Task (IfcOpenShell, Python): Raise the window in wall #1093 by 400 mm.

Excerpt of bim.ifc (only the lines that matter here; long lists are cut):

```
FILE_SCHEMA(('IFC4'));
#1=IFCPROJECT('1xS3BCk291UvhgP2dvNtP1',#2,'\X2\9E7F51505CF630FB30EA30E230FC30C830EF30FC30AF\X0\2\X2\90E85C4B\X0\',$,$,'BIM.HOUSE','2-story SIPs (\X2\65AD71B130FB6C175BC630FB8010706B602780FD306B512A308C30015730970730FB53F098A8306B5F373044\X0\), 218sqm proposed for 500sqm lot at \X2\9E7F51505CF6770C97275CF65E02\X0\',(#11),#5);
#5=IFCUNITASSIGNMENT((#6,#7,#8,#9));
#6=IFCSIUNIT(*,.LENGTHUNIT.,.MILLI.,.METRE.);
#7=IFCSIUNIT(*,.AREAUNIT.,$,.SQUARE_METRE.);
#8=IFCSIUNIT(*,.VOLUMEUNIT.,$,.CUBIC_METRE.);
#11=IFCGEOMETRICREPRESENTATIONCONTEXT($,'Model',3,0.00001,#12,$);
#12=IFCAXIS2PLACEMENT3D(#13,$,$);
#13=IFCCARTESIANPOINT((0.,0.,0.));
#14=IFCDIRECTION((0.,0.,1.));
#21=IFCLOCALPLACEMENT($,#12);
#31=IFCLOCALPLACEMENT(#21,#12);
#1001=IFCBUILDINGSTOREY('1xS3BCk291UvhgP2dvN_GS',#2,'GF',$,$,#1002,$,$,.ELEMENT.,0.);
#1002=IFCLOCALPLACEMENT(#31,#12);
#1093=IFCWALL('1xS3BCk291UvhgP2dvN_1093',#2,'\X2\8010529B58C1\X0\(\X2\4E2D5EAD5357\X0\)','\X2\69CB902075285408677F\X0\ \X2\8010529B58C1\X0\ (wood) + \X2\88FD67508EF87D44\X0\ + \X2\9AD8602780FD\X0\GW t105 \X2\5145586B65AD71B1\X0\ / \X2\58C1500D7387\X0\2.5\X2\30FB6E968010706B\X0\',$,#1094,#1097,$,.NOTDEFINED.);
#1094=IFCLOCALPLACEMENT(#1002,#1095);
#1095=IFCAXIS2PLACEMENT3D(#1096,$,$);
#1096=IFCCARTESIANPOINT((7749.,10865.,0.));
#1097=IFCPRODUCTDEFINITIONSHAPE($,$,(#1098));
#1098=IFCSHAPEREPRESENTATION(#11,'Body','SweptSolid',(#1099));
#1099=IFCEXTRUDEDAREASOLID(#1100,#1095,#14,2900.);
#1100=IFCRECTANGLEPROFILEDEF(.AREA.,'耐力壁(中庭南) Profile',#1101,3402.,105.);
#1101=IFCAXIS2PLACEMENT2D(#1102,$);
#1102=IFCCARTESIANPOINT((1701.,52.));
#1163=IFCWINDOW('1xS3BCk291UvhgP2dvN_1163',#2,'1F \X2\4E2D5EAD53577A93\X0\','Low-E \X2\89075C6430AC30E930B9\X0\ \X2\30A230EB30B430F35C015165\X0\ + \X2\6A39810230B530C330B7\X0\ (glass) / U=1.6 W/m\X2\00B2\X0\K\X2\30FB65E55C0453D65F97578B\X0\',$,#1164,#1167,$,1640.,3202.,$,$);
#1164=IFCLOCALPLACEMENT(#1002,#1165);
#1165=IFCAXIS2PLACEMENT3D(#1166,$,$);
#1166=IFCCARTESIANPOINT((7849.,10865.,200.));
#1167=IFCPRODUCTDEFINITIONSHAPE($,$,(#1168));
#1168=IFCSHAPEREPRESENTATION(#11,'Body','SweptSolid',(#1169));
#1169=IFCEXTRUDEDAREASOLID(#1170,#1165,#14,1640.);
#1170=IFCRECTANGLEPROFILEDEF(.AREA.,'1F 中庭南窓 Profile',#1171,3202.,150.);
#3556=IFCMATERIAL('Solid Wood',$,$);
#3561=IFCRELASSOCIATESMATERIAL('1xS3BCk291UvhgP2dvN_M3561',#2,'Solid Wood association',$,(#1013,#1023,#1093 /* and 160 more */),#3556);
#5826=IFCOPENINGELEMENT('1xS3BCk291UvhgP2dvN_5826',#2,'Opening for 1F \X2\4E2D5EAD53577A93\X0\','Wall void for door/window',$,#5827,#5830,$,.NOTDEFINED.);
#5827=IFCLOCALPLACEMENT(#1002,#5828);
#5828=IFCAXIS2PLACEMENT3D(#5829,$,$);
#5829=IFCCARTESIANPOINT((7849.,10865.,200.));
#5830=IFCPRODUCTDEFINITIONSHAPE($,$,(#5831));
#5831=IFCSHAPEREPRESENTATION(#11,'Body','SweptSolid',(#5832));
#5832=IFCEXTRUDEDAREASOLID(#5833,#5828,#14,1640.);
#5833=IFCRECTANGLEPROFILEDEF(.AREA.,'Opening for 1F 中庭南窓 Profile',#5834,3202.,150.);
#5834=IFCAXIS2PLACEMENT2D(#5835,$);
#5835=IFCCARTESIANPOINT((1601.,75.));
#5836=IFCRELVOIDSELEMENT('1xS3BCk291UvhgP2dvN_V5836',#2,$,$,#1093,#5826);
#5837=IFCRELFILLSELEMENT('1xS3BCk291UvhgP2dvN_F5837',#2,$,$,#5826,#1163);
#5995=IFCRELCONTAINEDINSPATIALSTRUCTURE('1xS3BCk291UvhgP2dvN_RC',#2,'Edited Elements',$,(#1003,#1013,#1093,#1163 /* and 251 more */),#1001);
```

```python
import numpy as np
import ifcopenshell
import ifcopenshell.api.geometry
import ifcopenshell.util.placement
import ifcopenshell.util.unit

model = ifcopenshell.open("bim.ifc")
unit_scale = ifcopenshell.util.unit.calculate_unit_scale(model)

window = model.by_guid("1xS3BCk291UvhgP2dvN_1163")
opening = window.FillsVoids[0].RelatingOpeningElement
dz = 0.4 / unit_scale

shift = np.array([0.0, 0.0, dz])
# The window is not placed relative to its opening, so move both.
for product in (opening, window):
    matrix = ifcopenshell.util.placement.get_local_placement(product.ObjectPlacement)
    matrix[:3, 3] += shift
    ifcopenshell.api.geometry.edit_object_placement(model, product=product, matrix=matrix, is_si=False)

print(f"moved by {dz * unit_scale:+.3f} m")

model.write("bim_v2.ifc")
```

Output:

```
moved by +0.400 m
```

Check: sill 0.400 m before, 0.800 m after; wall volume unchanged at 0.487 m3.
